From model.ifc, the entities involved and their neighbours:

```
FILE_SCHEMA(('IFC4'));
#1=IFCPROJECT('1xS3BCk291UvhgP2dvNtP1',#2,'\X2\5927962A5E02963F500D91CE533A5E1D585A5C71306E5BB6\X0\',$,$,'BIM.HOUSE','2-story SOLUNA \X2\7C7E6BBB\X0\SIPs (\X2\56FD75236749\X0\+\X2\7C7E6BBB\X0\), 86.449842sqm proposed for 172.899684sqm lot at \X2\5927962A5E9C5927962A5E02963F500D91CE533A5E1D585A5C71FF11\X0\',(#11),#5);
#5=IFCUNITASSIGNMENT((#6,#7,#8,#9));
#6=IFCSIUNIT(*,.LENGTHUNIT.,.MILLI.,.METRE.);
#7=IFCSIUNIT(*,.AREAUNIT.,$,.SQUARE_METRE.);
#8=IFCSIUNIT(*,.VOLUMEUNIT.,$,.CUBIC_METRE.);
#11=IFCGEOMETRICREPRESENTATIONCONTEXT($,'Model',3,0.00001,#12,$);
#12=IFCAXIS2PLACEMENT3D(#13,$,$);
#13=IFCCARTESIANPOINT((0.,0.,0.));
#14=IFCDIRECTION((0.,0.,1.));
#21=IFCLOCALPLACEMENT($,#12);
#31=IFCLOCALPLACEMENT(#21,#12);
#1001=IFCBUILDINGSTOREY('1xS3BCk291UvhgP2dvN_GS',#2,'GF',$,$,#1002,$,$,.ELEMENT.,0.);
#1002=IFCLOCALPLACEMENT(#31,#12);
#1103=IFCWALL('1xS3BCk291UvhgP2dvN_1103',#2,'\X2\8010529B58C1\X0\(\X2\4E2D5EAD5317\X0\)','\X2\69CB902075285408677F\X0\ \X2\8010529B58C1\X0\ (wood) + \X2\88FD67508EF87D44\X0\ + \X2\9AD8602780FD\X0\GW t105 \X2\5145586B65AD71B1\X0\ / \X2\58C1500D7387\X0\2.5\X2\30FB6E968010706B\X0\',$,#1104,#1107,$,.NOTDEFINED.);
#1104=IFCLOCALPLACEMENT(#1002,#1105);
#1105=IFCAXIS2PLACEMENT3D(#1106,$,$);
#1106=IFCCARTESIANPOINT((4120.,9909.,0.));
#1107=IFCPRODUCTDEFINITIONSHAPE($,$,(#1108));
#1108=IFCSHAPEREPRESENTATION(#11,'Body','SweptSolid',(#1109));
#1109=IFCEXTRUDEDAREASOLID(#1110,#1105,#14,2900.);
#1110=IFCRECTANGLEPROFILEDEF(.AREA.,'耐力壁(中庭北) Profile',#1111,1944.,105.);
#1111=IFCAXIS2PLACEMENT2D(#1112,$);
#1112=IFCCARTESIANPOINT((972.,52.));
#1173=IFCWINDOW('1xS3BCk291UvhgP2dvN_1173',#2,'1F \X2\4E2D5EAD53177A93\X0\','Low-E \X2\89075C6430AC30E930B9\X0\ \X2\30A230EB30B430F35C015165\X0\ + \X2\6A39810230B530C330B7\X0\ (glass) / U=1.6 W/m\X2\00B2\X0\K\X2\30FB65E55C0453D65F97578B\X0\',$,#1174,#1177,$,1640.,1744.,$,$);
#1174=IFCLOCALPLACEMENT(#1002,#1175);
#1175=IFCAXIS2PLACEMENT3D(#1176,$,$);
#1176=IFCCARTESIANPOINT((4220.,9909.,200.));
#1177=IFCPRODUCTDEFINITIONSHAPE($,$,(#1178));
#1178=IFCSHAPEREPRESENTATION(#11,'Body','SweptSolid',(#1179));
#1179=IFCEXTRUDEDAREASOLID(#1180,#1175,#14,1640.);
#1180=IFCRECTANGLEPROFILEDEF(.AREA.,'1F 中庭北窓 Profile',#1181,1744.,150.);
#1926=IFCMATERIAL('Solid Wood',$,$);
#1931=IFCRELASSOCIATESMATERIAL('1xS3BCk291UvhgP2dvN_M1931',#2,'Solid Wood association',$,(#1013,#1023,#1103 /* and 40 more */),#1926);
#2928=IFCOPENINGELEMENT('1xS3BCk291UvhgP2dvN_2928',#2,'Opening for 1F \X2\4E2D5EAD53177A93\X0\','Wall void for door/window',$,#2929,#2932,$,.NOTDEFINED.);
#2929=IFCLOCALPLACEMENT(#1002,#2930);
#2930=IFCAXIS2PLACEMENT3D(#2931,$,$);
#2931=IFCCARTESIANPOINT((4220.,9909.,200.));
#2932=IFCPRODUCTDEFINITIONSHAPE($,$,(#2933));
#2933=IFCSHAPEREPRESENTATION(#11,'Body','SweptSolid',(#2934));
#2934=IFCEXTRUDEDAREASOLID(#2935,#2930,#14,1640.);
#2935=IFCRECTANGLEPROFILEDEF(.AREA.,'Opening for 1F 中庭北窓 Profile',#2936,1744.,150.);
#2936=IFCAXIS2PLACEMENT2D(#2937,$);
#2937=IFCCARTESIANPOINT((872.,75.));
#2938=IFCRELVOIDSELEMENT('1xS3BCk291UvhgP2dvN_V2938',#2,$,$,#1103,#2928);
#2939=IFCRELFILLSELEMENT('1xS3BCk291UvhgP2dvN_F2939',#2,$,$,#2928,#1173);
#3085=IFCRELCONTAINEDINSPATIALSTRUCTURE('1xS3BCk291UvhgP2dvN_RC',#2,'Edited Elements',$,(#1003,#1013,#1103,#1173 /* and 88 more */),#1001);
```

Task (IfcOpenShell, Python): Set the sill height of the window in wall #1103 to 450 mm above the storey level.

```python
import numpy as np
import ifcopenshell
import ifcopenshell.api.geometry
import ifcopenshell.geom
import ifcopenshell.util.element
import ifcopenshell.util.placement
import ifcopenshell.util.shape
import ifcopenshell.util.unit

model = ifcopenshell.open("model.ifc")
unit_scale = ifcopenshell.util.unit.calculate_unit_scale(model)

window = model.by_guid("1xS3BCk291UvhgP2dvN_1173")
opening = window.FillsVoids[0].RelatingOpeningElement
storey = ifcopenshell.util.element.get_container(window, ifc_class="IfcBuildingStorey")
level = ifcopenshell.util.placement.get_local_placement(storey.ObjectPlacement)[2, 3]

# The opening's origin need not be at the sill, so measure its lowest point.
shape = ifcopenshell.geom.create_shape(ifcopenshell.geom.settings(), opening)
bottom = ifcopenshell.util.shape.get_shape_bottom_elevation(shape, shape.geometry) / unit_scale
dz = level + 0.45 / unit_scale - bottom

shift = np.array([0.0, 0.0, dz])
# The window is not placed relative to its opening, so move both.
for product in (opening, window):
    matrix = ifcopenshell.util.placement.get_local_placement(product.ObjectPlacement)
    matrix[:3, 3] += shift
    ifcopenshell.api.geometry.edit_object_placement(model, product=product, matrix=matrix, is_si=False)

print(f"moved by {dz * unit_scale:+.3f} m")

model.write("model_rev.ifc")
```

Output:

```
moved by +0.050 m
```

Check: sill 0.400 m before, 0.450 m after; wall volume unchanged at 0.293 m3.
